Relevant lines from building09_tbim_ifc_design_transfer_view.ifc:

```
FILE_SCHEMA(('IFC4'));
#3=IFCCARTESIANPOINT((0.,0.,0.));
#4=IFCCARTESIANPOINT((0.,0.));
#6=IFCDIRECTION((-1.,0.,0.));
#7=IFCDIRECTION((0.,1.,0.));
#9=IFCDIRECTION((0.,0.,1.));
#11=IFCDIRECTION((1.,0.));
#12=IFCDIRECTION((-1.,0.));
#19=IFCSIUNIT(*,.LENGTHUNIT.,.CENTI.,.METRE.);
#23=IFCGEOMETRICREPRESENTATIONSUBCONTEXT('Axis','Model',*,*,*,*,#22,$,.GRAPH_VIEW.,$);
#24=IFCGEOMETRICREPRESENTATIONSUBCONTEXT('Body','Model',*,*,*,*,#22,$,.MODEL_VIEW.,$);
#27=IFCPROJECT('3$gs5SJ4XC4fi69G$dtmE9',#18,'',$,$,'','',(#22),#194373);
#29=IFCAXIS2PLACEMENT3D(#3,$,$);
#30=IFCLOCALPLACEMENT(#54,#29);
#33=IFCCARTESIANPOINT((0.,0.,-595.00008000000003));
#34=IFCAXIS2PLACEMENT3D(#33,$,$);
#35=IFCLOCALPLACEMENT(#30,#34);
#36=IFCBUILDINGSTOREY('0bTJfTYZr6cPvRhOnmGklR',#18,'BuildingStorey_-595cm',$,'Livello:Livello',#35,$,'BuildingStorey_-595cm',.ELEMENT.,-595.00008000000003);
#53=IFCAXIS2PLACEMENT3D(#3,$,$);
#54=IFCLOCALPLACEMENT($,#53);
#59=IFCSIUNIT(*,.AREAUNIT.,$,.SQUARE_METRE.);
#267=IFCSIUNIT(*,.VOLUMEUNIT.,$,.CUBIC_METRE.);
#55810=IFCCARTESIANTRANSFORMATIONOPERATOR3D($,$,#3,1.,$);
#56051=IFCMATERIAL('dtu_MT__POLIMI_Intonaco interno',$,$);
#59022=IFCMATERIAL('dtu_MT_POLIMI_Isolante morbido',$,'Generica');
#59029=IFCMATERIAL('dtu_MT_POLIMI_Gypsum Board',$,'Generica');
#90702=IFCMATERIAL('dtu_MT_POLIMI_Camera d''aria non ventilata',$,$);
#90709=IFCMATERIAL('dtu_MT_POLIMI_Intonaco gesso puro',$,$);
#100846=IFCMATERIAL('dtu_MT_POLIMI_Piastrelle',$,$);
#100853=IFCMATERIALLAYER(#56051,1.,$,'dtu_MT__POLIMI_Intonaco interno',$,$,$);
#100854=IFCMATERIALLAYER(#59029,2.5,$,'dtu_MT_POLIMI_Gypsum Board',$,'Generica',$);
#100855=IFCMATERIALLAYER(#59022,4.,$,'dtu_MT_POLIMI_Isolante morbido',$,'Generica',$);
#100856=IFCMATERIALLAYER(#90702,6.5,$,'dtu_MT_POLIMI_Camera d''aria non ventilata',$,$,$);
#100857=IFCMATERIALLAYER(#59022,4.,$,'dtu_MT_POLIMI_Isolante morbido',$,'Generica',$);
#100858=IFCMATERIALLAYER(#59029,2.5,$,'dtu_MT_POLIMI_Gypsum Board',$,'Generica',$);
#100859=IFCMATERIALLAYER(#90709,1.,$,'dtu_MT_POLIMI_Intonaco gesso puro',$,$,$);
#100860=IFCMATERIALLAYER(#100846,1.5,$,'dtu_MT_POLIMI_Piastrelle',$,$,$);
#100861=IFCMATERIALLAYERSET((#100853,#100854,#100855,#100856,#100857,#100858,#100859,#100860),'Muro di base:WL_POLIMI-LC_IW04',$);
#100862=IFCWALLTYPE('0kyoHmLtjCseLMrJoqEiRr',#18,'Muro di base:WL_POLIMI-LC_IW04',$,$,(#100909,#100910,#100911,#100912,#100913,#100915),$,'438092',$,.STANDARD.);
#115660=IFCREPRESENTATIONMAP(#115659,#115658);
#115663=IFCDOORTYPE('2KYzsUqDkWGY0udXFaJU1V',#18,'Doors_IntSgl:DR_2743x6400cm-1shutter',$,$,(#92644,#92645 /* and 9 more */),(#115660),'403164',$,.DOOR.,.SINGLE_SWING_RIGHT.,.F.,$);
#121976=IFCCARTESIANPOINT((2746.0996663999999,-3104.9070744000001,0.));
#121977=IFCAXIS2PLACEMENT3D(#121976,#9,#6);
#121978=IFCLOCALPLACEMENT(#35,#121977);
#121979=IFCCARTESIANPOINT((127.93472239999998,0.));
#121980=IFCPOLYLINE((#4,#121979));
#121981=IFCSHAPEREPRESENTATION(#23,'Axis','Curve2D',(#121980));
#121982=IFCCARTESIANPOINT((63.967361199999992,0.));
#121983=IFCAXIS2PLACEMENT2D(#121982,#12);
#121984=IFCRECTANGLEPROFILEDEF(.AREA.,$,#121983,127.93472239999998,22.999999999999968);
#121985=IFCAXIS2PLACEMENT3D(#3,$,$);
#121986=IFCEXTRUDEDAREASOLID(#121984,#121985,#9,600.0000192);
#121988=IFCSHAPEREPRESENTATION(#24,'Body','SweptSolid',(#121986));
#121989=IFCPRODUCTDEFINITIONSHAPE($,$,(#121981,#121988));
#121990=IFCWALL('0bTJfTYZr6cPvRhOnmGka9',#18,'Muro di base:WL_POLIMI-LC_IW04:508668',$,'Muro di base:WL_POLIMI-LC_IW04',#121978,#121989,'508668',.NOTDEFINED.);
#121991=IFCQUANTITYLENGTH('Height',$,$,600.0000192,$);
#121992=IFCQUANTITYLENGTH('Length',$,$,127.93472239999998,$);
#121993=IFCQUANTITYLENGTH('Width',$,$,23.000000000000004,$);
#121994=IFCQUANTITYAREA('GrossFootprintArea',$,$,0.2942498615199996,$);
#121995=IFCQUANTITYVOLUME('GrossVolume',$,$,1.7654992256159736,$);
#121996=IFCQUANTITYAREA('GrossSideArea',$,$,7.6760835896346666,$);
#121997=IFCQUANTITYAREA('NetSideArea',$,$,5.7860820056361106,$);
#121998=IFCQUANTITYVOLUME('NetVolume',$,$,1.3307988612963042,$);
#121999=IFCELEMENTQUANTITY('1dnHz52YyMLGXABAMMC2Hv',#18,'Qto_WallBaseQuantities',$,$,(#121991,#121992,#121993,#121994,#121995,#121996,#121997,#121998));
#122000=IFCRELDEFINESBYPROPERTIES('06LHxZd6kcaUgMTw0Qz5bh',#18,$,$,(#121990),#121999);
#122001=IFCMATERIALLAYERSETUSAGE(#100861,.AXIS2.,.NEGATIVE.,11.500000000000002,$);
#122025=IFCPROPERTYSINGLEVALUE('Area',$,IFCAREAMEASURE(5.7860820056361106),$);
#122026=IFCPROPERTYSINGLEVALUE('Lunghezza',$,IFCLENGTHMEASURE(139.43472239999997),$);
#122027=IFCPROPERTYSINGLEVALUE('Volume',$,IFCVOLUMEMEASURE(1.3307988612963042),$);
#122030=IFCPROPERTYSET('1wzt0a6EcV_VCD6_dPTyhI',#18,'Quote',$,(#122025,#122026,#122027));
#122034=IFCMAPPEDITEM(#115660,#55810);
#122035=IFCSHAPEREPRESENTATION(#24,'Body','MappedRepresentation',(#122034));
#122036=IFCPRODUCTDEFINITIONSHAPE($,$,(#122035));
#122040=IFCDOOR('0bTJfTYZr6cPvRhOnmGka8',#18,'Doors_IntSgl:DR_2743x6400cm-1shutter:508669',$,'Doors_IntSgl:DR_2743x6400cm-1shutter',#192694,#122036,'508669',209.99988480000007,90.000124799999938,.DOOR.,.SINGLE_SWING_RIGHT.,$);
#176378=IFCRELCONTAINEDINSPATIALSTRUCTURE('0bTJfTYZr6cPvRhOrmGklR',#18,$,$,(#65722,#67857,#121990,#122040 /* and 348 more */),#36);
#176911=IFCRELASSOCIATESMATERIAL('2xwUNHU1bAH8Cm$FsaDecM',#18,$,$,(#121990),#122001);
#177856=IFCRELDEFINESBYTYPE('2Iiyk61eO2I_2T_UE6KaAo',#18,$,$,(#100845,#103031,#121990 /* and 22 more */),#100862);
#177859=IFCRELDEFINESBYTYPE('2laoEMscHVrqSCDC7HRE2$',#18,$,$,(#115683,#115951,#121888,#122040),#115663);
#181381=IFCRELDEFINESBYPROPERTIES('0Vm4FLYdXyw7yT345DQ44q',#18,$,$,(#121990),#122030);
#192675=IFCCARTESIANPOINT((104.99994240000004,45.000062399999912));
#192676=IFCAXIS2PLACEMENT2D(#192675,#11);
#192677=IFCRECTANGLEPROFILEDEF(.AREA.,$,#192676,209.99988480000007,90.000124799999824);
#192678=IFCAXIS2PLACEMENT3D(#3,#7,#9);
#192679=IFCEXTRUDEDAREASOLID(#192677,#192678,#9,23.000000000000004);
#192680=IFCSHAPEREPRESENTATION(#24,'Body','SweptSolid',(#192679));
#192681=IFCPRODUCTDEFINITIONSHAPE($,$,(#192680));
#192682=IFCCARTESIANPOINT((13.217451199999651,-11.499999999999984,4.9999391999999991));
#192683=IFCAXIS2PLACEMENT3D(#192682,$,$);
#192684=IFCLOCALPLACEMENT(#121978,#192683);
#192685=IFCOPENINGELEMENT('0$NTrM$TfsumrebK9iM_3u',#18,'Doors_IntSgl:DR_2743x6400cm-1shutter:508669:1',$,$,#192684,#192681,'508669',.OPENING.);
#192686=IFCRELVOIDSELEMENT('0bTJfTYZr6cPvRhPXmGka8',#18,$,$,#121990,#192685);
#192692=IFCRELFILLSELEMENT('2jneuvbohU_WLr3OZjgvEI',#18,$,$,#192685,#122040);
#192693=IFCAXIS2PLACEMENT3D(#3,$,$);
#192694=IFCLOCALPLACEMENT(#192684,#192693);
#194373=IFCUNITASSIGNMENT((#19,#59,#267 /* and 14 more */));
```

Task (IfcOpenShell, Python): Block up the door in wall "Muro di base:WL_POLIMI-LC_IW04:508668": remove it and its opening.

```python
import ifcopenshell
import ifcopenshell.api.feature
import ifcopenshell.api.pset
import ifcopenshell.api.root
import ifcopenshell.geom
import ifcopenshell.util.element
import ifcopenshell.util.shape
import ifcopenshell.util.unit

model = ifcopenshell.open("building09_tbim_ifc_design_transfer_view.ifc")
area_scale = ifcopenshell.util.unit.calculate_unit_scale(model, "AREAUNIT")
volume_scale = ifcopenshell.util.unit.calculate_unit_scale(model, "VOLUMEUNIT")
settings = ifcopenshell.geom.settings()


def volume(element):
    """Net volume in cubic metres, openings subtracted."""
    shape = ifcopenshell.geom.create_shape(settings, element)
    return ifcopenshell.util.shape.get_volume(shape.geometry)


door = model.by_guid("0bTJfTYZr6cPvRhOnmGka8")
opening = door.FillsVoids[0].RelatingOpeningElement
wall = opening.VoidsElements[0].RelatingBuildingElement
before = volume(wall)

ifcopenshell.api.root.remove_product(model, product=door)
ifcopenshell.api.feature.remove_feature(model, feature=opening)

after = volume(wall)
thickness = 0.23  # wall thickness in metres

# Update the wall's stored quantities.
qto = model.by_id(ifcopenshell.util.element.get_pset(wall, "Qto_WallBaseQuantities", should_inherit=False)["id"])
ifcopenshell.api.pset.edit_qto(model, qto=qto, properties={
    "NetSideArea": after / thickness / area_scale,
    "NetVolume": after / volume_scale,
})
pset = model.by_id(ifcopenshell.util.element.get_pset(wall, "Quote", should_inherit=False)["id"])
ifcopenshell.api.pset.edit_pset(model, pset=pset, properties={
    "Area": model.create_entity("IfcAreaMeasure", after / thickness / area_scale),
    "Volume": model.create_entity("IfcVolumeMeasure", after / volume_scale),
})

print(f"wall volume {before:.3f} -> {after:.3f} m3")

model.write("building09_tbim_ifc_design_transfer_view_v2.ifc")
```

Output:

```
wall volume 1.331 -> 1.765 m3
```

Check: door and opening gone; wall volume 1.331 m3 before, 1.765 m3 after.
